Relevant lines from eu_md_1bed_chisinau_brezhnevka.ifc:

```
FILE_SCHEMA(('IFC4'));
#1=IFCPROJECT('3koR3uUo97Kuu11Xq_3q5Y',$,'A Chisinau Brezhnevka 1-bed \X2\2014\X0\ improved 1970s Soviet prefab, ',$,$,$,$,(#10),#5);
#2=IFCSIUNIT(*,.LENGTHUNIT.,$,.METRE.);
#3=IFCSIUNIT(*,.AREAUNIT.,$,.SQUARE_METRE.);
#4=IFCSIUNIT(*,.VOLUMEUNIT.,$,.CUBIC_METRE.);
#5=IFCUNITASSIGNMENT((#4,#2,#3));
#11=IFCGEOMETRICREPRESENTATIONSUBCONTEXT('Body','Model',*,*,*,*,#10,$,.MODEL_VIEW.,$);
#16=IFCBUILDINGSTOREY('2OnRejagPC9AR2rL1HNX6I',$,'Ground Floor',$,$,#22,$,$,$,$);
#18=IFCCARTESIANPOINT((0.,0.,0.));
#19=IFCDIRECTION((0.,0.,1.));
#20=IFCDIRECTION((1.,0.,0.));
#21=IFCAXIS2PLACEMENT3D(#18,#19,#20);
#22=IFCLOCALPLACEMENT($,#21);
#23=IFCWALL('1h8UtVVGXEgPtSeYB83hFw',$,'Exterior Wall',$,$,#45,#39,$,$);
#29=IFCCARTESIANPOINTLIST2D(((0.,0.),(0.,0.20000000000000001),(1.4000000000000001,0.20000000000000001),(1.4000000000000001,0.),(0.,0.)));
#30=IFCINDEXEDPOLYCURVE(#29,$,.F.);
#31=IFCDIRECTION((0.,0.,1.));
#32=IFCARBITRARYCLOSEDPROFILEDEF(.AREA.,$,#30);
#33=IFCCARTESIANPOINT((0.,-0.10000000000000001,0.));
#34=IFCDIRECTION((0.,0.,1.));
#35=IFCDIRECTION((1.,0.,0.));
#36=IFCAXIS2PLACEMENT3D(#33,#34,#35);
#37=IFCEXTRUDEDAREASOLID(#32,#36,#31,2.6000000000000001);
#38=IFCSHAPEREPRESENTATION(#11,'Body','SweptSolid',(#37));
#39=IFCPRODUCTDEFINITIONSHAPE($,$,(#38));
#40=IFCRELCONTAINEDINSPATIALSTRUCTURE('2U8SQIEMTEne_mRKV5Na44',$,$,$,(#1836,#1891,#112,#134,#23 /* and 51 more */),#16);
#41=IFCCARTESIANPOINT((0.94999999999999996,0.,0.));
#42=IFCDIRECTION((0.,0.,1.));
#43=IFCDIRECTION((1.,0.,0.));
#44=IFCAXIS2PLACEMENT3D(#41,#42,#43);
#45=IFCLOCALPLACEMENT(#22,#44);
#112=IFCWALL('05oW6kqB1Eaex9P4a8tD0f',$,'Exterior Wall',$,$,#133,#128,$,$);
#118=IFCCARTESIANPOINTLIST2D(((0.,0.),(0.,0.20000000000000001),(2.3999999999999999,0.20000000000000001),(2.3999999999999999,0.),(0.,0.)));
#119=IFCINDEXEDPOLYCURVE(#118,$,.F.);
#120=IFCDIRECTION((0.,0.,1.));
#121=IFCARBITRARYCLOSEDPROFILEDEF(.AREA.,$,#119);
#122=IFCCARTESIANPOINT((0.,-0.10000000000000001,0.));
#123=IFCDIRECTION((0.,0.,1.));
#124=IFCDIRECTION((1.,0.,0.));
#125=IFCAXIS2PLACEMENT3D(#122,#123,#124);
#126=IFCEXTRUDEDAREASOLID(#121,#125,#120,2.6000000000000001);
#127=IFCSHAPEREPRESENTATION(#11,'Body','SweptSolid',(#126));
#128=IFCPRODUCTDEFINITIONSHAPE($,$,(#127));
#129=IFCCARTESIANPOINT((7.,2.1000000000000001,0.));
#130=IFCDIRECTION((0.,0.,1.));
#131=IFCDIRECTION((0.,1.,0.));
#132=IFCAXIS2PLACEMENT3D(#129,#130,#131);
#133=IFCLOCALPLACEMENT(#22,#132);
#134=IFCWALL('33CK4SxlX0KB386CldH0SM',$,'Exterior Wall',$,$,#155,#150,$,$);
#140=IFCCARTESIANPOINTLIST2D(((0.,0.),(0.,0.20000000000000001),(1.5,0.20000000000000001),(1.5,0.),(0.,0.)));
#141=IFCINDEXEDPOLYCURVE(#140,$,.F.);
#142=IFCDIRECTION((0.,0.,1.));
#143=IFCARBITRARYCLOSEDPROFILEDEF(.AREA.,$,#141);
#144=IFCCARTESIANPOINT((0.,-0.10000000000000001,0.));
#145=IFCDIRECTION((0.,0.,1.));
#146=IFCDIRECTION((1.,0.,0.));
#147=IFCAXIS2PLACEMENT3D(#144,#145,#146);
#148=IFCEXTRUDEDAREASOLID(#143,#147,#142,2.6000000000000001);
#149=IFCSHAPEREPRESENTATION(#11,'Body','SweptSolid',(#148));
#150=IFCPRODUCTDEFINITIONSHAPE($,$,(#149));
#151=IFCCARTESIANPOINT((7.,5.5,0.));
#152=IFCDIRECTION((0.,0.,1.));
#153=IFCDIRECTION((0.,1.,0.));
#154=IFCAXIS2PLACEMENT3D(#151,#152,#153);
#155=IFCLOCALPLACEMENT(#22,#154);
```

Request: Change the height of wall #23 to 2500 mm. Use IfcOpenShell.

```python
import ifcopenshell
import ifcopenshell.geom
import ifcopenshell.util.representation
import ifcopenshell.util.shape
import ifcopenshell.util.unit

model = ifcopenshell.open("eu_md_1bed_chisinau_brezhnevka.ifc")
unit_scale = ifcopenshell.util.unit.calculate_unit_scale(model)
settings = ifcopenshell.geom.settings()


def volume(element):
    """Net volume in cubic metres, openings subtracted."""
    shape = ifcopenshell.geom.create_shape(settings, element)
    return ifcopenshell.util.shape.get_volume(shape.geometry)


wall = model.by_guid("1h8UtVVGXEgPtSeYB83hFw")
before = volume(wall)

body = ifcopenshell.util.representation.get_representation(wall, "Model", "Body")
solid = body.Items[0]
old_height = solid.Depth
solid.Depth = 2.5 / unit_scale
after = volume(wall)

print(f"height {old_height:g} -> {solid.Depth:g}, volume {before:.3f} -> {after:.3f} m3")

model.write("eu_md_1bed_chisinau_brezhnevka_rev.ifc")
```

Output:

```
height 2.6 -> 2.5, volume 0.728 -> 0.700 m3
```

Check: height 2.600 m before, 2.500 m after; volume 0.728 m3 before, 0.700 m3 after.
